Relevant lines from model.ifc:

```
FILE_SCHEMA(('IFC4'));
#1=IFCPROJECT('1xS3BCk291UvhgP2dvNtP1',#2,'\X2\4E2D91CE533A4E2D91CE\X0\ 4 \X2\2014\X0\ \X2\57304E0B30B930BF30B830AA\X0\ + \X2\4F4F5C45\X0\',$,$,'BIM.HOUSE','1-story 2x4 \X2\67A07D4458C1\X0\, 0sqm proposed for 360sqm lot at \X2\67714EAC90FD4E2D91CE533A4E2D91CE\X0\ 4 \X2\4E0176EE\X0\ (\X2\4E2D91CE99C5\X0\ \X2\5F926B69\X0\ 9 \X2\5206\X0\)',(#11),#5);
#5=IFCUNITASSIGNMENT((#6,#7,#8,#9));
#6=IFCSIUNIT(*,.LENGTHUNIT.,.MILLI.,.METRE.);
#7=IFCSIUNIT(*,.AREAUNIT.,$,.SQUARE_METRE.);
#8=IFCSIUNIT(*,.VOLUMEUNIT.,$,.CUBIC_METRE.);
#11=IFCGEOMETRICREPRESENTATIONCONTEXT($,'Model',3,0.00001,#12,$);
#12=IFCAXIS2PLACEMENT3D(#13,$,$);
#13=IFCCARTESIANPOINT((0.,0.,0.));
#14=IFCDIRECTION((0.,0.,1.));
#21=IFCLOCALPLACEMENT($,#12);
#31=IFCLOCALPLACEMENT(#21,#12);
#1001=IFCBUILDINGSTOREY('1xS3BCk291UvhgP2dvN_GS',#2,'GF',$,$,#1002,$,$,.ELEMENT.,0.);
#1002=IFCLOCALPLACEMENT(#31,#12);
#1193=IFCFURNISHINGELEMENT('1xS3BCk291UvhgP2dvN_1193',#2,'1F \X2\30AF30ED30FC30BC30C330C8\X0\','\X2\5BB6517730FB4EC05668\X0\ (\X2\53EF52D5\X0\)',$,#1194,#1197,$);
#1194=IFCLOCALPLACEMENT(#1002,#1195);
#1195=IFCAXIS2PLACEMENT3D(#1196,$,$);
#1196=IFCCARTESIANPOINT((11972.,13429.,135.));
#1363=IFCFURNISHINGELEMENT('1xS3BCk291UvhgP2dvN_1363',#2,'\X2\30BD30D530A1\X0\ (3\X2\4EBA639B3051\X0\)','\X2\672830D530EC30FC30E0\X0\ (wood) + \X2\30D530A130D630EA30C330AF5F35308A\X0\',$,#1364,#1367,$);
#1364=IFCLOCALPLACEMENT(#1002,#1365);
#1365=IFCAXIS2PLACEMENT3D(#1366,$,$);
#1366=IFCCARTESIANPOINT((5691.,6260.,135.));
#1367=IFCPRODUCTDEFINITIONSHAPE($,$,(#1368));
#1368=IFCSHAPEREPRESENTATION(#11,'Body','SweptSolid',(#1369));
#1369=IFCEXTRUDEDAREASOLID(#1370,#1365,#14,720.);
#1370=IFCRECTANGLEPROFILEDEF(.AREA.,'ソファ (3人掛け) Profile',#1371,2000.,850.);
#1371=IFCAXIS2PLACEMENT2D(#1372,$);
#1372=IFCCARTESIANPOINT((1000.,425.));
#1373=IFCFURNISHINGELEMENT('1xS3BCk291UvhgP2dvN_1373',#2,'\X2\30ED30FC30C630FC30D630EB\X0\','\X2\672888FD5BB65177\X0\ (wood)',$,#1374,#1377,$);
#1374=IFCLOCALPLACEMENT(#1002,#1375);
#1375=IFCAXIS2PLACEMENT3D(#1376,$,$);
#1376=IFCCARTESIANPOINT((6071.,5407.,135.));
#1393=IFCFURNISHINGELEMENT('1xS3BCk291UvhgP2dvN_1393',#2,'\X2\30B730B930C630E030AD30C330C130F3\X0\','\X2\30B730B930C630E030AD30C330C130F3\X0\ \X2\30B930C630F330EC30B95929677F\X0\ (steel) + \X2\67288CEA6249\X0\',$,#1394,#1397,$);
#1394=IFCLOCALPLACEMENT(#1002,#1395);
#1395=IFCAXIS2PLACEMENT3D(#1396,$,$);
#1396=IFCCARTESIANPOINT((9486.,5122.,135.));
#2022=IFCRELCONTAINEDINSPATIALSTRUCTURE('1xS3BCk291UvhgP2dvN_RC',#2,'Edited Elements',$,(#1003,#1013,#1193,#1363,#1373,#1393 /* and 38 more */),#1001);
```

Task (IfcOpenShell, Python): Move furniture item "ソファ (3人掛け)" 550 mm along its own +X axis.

```python
import ifcopenshell
import ifcopenshell.api.geometry
import ifcopenshell.util.placement

model = ifcopenshell.open("model.ifc")

item = model.by_guid("1xS3BCk291UvhgP2dvN_1363")
matrix = ifcopenshell.util.placement.get_local_placement(item.ObjectPlacement)
matrix[:3, 3] += matrix[:3, 0] * 550.0
ifcopenshell.api.geometry.edit_object_placement(model, product=item, matrix=matrix, is_si=False)

print(ifcopenshell.util.placement.get_local_placement(item.ObjectPlacement).round(3) + 0.0)

model.write("model_updated.ifc")
```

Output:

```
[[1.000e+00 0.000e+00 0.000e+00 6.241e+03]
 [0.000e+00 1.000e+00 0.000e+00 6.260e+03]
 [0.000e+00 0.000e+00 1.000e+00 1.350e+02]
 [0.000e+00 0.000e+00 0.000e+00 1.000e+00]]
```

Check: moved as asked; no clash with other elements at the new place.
